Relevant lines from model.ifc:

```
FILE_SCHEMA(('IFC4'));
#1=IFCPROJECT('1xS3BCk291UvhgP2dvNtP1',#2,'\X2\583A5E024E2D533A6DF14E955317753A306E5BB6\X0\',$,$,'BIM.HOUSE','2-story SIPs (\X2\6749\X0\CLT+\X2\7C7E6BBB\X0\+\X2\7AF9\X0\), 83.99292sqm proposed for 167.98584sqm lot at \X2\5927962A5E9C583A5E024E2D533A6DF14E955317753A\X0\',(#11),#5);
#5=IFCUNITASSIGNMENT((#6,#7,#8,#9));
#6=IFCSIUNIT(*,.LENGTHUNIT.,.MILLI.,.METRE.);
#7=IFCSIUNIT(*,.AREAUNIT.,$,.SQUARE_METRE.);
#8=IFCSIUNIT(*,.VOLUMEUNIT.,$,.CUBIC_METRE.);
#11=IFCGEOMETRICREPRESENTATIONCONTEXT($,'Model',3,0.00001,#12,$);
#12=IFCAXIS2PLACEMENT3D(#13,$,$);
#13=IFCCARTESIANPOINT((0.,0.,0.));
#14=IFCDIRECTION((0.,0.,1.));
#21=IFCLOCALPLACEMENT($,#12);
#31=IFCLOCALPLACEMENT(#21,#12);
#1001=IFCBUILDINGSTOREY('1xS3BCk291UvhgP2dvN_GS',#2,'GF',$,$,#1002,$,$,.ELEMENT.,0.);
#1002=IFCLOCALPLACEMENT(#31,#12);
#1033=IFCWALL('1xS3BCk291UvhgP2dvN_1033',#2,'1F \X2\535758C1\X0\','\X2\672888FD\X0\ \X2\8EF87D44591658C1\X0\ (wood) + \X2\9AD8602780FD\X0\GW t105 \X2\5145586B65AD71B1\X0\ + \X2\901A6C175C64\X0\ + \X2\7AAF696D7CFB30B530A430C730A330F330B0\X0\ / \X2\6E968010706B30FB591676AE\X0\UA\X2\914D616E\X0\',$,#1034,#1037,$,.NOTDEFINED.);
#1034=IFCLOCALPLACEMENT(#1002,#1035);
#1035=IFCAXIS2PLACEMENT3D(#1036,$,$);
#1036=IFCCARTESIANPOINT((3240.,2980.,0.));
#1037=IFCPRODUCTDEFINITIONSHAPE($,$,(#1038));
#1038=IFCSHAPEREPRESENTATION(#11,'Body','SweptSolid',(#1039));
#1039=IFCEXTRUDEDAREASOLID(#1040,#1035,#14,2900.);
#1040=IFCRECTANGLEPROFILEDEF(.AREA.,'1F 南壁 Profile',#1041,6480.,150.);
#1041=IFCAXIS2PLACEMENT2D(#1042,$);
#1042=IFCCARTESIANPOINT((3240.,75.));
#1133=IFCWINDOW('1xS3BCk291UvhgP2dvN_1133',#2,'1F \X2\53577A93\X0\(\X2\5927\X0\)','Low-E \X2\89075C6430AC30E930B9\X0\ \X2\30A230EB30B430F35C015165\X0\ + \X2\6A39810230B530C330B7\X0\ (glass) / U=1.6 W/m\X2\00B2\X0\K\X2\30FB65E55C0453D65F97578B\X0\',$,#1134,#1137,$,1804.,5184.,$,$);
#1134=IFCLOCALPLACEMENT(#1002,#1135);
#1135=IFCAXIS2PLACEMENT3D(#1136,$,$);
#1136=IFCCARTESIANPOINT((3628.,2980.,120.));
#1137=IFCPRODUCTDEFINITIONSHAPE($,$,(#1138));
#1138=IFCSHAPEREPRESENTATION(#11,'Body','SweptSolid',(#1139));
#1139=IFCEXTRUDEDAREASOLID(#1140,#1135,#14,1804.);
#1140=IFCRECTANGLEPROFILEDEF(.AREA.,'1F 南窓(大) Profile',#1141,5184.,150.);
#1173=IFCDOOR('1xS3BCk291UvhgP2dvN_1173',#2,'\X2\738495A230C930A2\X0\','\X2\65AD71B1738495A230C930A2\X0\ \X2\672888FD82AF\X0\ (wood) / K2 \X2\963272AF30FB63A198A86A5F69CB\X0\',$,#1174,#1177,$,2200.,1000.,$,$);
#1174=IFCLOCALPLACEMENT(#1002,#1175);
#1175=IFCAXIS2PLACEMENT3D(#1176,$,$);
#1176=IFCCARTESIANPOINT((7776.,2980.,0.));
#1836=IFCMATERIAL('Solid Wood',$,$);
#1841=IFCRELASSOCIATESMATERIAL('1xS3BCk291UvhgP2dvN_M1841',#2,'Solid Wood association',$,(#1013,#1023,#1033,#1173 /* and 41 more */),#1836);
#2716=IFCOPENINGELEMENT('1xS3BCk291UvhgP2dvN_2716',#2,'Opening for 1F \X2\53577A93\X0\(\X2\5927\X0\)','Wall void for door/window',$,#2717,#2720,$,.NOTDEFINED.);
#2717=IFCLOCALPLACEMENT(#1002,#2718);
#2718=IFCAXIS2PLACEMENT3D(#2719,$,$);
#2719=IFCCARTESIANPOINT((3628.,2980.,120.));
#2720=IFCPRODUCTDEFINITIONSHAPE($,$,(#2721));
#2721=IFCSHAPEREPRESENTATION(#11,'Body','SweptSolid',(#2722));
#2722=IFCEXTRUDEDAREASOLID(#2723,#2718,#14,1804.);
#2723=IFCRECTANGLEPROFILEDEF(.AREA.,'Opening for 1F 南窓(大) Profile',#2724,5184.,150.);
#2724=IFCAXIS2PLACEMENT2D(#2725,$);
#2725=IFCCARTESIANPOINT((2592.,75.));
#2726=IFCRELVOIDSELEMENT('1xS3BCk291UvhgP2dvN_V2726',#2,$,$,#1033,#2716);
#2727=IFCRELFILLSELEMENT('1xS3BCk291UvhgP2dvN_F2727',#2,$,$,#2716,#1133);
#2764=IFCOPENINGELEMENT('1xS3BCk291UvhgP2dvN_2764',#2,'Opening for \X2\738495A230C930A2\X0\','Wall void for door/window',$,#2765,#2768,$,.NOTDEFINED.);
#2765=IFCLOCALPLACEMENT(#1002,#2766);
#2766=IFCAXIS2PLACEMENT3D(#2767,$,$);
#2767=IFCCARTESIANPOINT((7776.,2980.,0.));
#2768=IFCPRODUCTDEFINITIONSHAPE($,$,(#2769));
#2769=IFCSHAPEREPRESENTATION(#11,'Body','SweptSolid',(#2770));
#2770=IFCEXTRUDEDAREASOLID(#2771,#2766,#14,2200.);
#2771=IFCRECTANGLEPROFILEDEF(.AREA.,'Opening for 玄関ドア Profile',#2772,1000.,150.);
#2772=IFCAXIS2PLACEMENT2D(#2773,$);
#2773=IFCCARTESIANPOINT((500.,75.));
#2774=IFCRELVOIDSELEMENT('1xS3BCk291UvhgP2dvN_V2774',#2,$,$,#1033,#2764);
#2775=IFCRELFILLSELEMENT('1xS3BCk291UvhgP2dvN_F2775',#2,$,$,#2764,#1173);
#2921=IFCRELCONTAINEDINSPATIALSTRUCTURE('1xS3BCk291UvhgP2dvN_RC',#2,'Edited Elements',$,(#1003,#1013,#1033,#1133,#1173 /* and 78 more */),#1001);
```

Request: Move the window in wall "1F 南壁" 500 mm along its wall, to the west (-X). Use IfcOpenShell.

```python
import ifcopenshell
import ifcopenshell.api.geometry
import ifcopenshell.util.placement

model = ifcopenshell.open("model.ifc")

window = model.by_guid("1xS3BCk291UvhgP2dvN_1133")
opening = window.FillsVoids[0].RelatingOpeningElement
wall = opening.VoidsElements[0].RelatingBuildingElement

wall_matrix = ifcopenshell.util.placement.get_local_placement(wall.ObjectPlacement)
shift = wall_matrix[:3, 0] * -500.0
before = ifcopenshell.util.placement.get_local_placement(window.ObjectPlacement)[:3, 3].copy()

# The window is not placed relative to its opening, so move both.
for product in (opening, window):
    matrix = ifcopenshell.util.placement.get_local_placement(product.ObjectPlacement)
    matrix[:3, 3] += shift
    ifcopenshell.api.geometry.edit_object_placement(model, product=product, matrix=matrix, is_si=False)

after = ifcopenshell.util.placement.get_local_placement(window.ObjectPlacement)[:3, 3]
print("window moved by", (after - before).round(3) + 0.0)

model.write("model_updated.ifc")
```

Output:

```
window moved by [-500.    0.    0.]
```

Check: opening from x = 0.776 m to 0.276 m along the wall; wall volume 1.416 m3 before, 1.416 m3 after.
